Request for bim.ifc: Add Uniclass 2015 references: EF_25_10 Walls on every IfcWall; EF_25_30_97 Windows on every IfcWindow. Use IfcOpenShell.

First a look at what the model holds.

```python
import ifcopenshell

model = ifcopenshell.open("bim.ifc")
print(model.schema)
print("classifications:", [c.Name for c in model.by_type("IfcClassification")])
for ifc_class in ("IfcDoor", "IfcRoof", "IfcStair", "IfcWall", "IfcWindow"):
    print(ifc_class, len(model.by_type(ifc_class)))
```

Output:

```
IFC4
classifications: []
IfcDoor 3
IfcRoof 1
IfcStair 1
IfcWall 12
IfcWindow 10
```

```python
import ifcopenshell
import ifcopenshell.api.classification

model = ifcopenshell.open("bim.ifc")

system = ifcopenshell.api.classification.add_classification(model, classification="Uniclass 2015")

codes = {
    "IfcWall": ("EF_25_10", "Walls"),
    "IfcWindow": ("EF_25_30_97", "Windows"),
}
for ifc_class, (code, name) in codes.items():
    products = model.by_type(ifc_class)
    ifcopenshell.api.classification.add_reference(
        model, products=products, classification=system, identification=code, name=name
    )
    print(code, len(products))

model.write("bim-out.ifc")
```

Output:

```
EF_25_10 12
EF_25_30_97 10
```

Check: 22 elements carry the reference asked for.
